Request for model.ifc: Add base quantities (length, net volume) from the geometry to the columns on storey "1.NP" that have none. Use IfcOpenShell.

First a look at what the model holds.

```python
import ifcopenshell
import ifcopenshell.util.element
import ifcopenshell.util.unit

model = ifcopenshell.open("model.ifc")
print(model.schema)
for unit_type in ("LENGTHUNIT", "AREAUNIT", "VOLUMEUNIT"):
    print(unit_type, ifcopenshell.util.unit.calculate_unit_scale(model, unit_type))
storey = next(s for s in model.by_type("IfcBuildingStorey") if s.Name == "1.NP")
columns = [e for e in ifcopenshell.util.element.get_decomposition(storey) if e.is_a("IfcColumn")]
for e in sorted(columns, key=lambda e: e.id()):
    print(e.id(), e.is_a(), e.Name, list(ifcopenshell.util.element.get_psets(e, qtos_only=True)), sep=" | ")
```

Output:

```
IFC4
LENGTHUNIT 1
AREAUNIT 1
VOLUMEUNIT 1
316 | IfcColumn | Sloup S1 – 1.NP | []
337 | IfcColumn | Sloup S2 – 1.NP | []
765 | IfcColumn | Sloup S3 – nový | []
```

```python
import ifcopenshell
import ifcopenshell.api.pset
import ifcopenshell.geom
import ifcopenshell.util.element
import ifcopenshell.util.shape
import ifcopenshell.util.unit

model = ifcopenshell.open("model.ifc")
unit_scale = ifcopenshell.util.unit.calculate_unit_scale(model)
volume_scale = ifcopenshell.util.unit.calculate_unit_scale(model, "VOLUMEUNIT")
settings = ifcopenshell.geom.settings()

storey = next(s for s in model.by_type("IfcBuildingStorey") if s.Name == "1.NP")
columns = [e for e in ifcopenshell.util.element.get_decomposition(storey) if e.is_a("IfcColumn")]

for e in sorted(columns, key=lambda e: e.id()):
    if ifcopenshell.util.element.get_psets(e, qtos_only=True, should_inherit=False):
        continue
    # Geometry comes back in metres, in the element's own axes.
    shape = ifcopenshell.geom.create_shape(settings, e)
    values = {
        "Length": ifcopenshell.util.shape.get_z(shape.geometry) / unit_scale,
        "NetVolume": ifcopenshell.util.shape.get_volume(shape.geometry) / volume_scale,
    }
    qto = ifcopenshell.api.pset.add_qto(model, product=e, name="Qto_ColumnBaseQuantities")
    ifcopenshell.api.pset.edit_qto(model, qto=qto, properties=values)
    print(e.id(), {k: round(v, 3) for k, v in values.items()})

model.write("model_v2.ifc")
```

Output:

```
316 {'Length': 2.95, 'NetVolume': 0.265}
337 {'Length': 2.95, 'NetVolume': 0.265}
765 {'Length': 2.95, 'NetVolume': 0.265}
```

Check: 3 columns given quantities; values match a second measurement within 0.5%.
